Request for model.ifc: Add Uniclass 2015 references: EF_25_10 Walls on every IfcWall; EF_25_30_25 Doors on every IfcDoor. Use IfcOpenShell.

First a look at what the model holds.

```python
import ifcopenshell

model = ifcopenshell.open("model.ifc")
print(model.schema)
print("classifications:", [c.Name for c in model.by_type("IfcClassification")])
for ifc_class in ("IfcDoor", "IfcRoof", "IfcStair", "IfcWall", "IfcWindow"):
    print(ifc_class, len(model.by_type(ifc_class)))
```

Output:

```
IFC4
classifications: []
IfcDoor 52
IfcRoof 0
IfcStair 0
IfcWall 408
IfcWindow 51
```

```python
import ifcopenshell
import ifcopenshell.api.classification

model = ifcopenshell.open("model.ifc")

system = ifcopenshell.api.classification.add_classification(model, classification="Uniclass 2015")

codes = {
    "IfcWall": ("EF_25_10", "Walls"),
    "IfcDoor": ("EF_25_30_25", "Doors"),
}
for ifc_class, (code, name) in codes.items():
    products = model.by_type(ifc_class)
    ifcopenshell.api.classification.add_reference(
        model, products=products, classification=system, identification=code, name=name
    )
    print(code, len(products))

model.write("model_v2.ifc")
```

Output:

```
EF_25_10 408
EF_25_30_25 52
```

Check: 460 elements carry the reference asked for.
